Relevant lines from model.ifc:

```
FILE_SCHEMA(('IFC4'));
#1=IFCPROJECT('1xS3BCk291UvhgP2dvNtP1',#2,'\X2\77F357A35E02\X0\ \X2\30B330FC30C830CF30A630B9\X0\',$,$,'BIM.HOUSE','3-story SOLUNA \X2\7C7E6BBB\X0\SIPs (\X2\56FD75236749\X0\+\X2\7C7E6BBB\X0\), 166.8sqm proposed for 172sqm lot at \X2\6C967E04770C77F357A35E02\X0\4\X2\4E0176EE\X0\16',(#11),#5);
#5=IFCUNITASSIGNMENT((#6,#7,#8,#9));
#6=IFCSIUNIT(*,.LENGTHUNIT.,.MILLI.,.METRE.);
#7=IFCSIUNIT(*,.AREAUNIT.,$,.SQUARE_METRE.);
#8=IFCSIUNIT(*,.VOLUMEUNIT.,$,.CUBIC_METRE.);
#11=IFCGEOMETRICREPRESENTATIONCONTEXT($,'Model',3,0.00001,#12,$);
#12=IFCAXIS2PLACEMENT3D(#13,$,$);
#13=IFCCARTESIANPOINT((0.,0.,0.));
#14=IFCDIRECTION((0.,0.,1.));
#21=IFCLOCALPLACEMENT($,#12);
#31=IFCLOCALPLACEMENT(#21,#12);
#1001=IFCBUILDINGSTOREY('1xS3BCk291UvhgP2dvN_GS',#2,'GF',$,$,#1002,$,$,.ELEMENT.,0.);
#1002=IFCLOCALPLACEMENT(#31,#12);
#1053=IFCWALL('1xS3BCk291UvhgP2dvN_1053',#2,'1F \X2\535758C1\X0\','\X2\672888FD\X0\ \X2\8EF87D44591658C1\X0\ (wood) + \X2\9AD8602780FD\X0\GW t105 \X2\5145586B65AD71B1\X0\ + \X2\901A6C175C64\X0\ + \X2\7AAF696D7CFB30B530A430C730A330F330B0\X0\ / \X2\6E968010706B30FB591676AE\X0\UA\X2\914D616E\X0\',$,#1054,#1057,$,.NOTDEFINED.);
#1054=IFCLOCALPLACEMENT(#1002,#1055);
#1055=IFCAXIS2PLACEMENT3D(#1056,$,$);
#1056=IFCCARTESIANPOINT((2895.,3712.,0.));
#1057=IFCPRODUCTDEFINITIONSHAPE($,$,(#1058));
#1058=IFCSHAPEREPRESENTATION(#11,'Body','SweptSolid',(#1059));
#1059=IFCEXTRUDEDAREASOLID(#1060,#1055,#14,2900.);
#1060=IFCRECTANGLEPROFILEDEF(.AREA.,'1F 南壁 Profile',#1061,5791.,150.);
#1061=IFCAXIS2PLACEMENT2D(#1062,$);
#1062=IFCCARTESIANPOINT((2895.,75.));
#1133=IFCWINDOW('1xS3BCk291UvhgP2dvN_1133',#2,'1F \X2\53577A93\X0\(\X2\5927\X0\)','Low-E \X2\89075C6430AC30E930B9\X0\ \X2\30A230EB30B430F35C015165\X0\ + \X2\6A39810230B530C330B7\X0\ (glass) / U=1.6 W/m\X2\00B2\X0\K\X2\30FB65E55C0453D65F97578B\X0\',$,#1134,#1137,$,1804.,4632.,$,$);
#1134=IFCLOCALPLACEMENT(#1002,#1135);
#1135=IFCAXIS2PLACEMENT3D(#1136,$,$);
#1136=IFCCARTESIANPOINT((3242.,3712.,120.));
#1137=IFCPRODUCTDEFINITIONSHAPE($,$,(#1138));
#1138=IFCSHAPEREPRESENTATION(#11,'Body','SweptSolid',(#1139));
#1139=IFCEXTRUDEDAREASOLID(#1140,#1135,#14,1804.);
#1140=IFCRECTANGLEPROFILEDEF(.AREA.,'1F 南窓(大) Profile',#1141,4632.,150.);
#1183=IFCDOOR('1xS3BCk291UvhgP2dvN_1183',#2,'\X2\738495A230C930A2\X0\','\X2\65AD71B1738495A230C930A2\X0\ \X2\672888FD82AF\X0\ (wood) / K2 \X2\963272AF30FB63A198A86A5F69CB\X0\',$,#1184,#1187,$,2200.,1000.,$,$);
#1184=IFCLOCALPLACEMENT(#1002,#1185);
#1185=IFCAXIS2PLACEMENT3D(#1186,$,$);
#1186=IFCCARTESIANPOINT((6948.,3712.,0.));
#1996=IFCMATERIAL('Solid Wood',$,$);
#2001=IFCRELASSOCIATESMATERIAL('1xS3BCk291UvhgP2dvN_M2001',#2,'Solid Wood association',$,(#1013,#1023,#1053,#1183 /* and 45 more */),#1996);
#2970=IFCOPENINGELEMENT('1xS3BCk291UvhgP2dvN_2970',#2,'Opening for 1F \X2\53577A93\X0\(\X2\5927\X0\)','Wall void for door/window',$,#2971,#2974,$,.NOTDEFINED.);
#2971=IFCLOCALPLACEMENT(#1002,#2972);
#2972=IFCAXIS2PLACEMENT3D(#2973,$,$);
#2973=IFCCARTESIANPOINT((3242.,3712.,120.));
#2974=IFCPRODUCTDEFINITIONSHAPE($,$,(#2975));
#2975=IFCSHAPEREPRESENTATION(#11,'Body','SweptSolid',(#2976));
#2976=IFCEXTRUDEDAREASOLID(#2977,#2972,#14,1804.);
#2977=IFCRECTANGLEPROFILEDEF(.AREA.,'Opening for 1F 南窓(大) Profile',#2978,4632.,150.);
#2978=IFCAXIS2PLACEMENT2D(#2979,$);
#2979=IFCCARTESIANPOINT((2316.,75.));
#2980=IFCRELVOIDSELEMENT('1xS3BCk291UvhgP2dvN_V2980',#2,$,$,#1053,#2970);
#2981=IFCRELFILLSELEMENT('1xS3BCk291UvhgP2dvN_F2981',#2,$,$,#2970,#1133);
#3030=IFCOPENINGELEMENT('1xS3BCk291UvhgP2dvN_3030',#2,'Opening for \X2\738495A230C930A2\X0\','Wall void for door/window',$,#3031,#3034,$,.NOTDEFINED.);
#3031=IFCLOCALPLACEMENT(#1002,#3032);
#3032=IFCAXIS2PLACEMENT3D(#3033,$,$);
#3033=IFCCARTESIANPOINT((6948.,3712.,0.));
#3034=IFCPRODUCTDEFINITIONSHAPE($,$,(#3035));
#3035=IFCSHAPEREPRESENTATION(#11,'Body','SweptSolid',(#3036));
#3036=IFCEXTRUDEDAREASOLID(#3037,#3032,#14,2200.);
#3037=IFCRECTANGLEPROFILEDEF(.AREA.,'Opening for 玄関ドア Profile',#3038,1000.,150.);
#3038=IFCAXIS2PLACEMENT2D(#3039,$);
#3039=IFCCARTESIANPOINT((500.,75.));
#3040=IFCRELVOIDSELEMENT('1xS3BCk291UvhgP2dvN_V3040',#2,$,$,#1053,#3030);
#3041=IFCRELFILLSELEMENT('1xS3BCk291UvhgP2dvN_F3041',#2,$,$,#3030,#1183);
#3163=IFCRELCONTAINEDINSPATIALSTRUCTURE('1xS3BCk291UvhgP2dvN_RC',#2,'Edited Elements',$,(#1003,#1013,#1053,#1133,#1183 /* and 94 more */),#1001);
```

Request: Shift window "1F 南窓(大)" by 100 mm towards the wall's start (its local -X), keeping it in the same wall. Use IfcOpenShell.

```python
import ifcopenshell
import ifcopenshell.api.geometry
import ifcopenshell.util.placement
import ifcopenshell.util.unit

model = ifcopenshell.open("model.ifc")
unit_scale = ifcopenshell.util.unit.calculate_unit_scale(model)

window = model.by_guid("1xS3BCk291UvhgP2dvN_1133")
opening = window.FillsVoids[0].RelatingOpeningElement
wall = opening.VoidsElements[0].RelatingBuildingElement

wall_matrix = ifcopenshell.util.placement.get_local_placement(wall.ObjectPlacement)
shift = wall_matrix[:3, 0] * -0.1 / unit_scale
before = ifcopenshell.util.placement.get_local_placement(window.ObjectPlacement)[:3, 3].copy()

# The window is not placed relative to its opening, so move both.
for product in (opening, window):
    matrix = ifcopenshell.util.placement.get_local_placement(product.ObjectPlacement)
    matrix[:3, 3] += shift
    ifcopenshell.api.geometry.edit_object_placement(model, product=product, matrix=matrix, is_si=False)

after = ifcopenshell.util.placement.get_local_placement(window.ObjectPlacement)[:3, 3]
print("window moved by", (after - before).round(3) + 0.0)

model.write("model_updated.ifc")
```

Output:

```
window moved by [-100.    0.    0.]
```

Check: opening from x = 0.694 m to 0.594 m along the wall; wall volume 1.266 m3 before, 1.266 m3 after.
